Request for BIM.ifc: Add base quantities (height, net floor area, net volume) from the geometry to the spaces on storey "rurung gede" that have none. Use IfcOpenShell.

First a look at what the model holds.

```python
import ifcopenshell
import ifcopenshell.util.element
import ifcopenshell.util.unit

model = ifcopenshell.open("BIM.ifc")
print(model.schema)
for unit_type in ("LENGTHUNIT", "AREAUNIT", "VOLUMEUNIT"):
    print(unit_type, ifcopenshell.util.unit.calculate_unit_scale(model, unit_type))
storey = next(s for s in model.by_type("IfcBuildingStorey") if s.Name == "rurung gede")
spaces = [e for e in ifcopenshell.util.element.get_decomposition(storey) if e.is_a("IfcSpace")]
for e in sorted(spaces, key=lambda e: e.id()):
    print(e.id(), e.is_a(), e.Name, list(ifcopenshell.util.element.get_psets(e, qtos_only=True)), sep=" | ")
```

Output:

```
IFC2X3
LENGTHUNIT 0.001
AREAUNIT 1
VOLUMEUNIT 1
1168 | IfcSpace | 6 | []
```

```python
import ifcopenshell
import ifcopenshell.api.pset
import ifcopenshell.geom
import ifcopenshell.util.element
import ifcopenshell.util.shape
import ifcopenshell.util.unit

model = ifcopenshell.open("BIM.ifc")
unit_scale = ifcopenshell.util.unit.calculate_unit_scale(model)
area_scale = ifcopenshell.util.unit.calculate_unit_scale(model, "AREAUNIT")
volume_scale = ifcopenshell.util.unit.calculate_unit_scale(model, "VOLUMEUNIT")
settings = ifcopenshell.geom.settings()

storey = next(s for s in model.by_type("IfcBuildingStorey") if s.Name == "rurung gede")
spaces = [e for e in ifcopenshell.util.element.get_decomposition(storey) if e.is_a("IfcSpace")]

for e in sorted(spaces, key=lambda e: e.id()):
    if ifcopenshell.util.element.get_psets(e, qtos_only=True, should_inherit=False):
        continue
    # Geometry comes back in metres, in the element's own axes.
    shape = ifcopenshell.geom.create_shape(settings, e)
    values = {
        "Height": ifcopenshell.util.shape.get_z(shape.geometry) / unit_scale,
        "NetFloorArea": ifcopenshell.util.shape.get_footprint_area(shape.geometry) / area_scale,
        "NetVolume": ifcopenshell.util.shape.get_volume(shape.geometry) / volume_scale,
    }
    qto = ifcopenshell.api.pset.add_qto(model, product=e, name="BaseQuantities")
    ifcopenshell.api.pset.edit_qto(model, qto=qto, properties=values)
    print(e.id(), {k: round(v, 3) for k, v in values.items()})

model.write("BIM_v2.ifc")
```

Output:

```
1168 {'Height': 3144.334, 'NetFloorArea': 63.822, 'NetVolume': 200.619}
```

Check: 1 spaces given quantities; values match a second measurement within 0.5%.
